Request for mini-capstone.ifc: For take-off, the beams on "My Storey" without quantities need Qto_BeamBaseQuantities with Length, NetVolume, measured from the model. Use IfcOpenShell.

First a look at what the model holds.

```python
import ifcopenshell
import ifcopenshell.util.element
import ifcopenshell.util.unit

model = ifcopenshell.open("mini-capstone.ifc")
print(model.schema)
for unit_type in ("LENGTHUNIT", "AREAUNIT", "VOLUMEUNIT"):
    print(unit_type, ifcopenshell.util.unit.calculate_unit_scale(model, unit_type))
storey = next(s for s in model.by_type("IfcBuildingStorey") if s.Name == "My Storey")
beams = [e for e in ifcopenshell.util.element.get_decomposition(storey) if e.is_a("IfcBeam")]
for e in sorted(beams, key=lambda e: e.id()):
    print(e.id(), e.is_a(), e.Name, list(ifcopenshell.util.element.get_psets(e, qtos_only=True)), sep=" | ")
```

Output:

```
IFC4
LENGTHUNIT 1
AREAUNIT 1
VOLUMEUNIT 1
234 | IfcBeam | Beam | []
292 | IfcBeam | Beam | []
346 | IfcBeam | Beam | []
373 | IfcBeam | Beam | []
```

```python
import ifcopenshell
import ifcopenshell.api.pset
import ifcopenshell.geom
import ifcopenshell.util.element
import ifcopenshell.util.shape
import ifcopenshell.util.unit

model = ifcopenshell.open("mini-capstone.ifc")
unit_scale = ifcopenshell.util.unit.calculate_unit_scale(model)
volume_scale = ifcopenshell.util.unit.calculate_unit_scale(model, "VOLUMEUNIT")
settings = ifcopenshell.geom.settings()

storey = next(s for s in model.by_type("IfcBuildingStorey") if s.Name == "My Storey")
beams = [e for e in ifcopenshell.util.element.get_decomposition(storey) if e.is_a("IfcBeam")]

for e in sorted(beams, key=lambda e: e.id()):
    if ifcopenshell.util.element.get_psets(e, qtos_only=True, should_inherit=False):
        continue
    # Geometry comes back in metres, in the element's own axes.
    shape = ifcopenshell.geom.create_shape(settings, e)
    values = {
        "Length": ifcopenshell.util.shape.get_max_xyz(shape.geometry) / unit_scale,
        "NetVolume": ifcopenshell.util.shape.get_volume(shape.geometry) / volume_scale,
    }
    qto = ifcopenshell.api.pset.add_qto(model, product=e, name="Qto_BeamBaseQuantities")
    ifcopenshell.api.pset.edit_qto(model, qto=qto, properties=values)
    print(e.id(), {k: round(v, 3) for k, v in values.items()})

model.write("mini-capstone-out.ifc")
```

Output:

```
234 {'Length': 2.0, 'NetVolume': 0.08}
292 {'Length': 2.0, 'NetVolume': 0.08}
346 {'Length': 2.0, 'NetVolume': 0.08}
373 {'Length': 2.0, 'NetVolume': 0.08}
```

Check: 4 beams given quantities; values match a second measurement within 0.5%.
